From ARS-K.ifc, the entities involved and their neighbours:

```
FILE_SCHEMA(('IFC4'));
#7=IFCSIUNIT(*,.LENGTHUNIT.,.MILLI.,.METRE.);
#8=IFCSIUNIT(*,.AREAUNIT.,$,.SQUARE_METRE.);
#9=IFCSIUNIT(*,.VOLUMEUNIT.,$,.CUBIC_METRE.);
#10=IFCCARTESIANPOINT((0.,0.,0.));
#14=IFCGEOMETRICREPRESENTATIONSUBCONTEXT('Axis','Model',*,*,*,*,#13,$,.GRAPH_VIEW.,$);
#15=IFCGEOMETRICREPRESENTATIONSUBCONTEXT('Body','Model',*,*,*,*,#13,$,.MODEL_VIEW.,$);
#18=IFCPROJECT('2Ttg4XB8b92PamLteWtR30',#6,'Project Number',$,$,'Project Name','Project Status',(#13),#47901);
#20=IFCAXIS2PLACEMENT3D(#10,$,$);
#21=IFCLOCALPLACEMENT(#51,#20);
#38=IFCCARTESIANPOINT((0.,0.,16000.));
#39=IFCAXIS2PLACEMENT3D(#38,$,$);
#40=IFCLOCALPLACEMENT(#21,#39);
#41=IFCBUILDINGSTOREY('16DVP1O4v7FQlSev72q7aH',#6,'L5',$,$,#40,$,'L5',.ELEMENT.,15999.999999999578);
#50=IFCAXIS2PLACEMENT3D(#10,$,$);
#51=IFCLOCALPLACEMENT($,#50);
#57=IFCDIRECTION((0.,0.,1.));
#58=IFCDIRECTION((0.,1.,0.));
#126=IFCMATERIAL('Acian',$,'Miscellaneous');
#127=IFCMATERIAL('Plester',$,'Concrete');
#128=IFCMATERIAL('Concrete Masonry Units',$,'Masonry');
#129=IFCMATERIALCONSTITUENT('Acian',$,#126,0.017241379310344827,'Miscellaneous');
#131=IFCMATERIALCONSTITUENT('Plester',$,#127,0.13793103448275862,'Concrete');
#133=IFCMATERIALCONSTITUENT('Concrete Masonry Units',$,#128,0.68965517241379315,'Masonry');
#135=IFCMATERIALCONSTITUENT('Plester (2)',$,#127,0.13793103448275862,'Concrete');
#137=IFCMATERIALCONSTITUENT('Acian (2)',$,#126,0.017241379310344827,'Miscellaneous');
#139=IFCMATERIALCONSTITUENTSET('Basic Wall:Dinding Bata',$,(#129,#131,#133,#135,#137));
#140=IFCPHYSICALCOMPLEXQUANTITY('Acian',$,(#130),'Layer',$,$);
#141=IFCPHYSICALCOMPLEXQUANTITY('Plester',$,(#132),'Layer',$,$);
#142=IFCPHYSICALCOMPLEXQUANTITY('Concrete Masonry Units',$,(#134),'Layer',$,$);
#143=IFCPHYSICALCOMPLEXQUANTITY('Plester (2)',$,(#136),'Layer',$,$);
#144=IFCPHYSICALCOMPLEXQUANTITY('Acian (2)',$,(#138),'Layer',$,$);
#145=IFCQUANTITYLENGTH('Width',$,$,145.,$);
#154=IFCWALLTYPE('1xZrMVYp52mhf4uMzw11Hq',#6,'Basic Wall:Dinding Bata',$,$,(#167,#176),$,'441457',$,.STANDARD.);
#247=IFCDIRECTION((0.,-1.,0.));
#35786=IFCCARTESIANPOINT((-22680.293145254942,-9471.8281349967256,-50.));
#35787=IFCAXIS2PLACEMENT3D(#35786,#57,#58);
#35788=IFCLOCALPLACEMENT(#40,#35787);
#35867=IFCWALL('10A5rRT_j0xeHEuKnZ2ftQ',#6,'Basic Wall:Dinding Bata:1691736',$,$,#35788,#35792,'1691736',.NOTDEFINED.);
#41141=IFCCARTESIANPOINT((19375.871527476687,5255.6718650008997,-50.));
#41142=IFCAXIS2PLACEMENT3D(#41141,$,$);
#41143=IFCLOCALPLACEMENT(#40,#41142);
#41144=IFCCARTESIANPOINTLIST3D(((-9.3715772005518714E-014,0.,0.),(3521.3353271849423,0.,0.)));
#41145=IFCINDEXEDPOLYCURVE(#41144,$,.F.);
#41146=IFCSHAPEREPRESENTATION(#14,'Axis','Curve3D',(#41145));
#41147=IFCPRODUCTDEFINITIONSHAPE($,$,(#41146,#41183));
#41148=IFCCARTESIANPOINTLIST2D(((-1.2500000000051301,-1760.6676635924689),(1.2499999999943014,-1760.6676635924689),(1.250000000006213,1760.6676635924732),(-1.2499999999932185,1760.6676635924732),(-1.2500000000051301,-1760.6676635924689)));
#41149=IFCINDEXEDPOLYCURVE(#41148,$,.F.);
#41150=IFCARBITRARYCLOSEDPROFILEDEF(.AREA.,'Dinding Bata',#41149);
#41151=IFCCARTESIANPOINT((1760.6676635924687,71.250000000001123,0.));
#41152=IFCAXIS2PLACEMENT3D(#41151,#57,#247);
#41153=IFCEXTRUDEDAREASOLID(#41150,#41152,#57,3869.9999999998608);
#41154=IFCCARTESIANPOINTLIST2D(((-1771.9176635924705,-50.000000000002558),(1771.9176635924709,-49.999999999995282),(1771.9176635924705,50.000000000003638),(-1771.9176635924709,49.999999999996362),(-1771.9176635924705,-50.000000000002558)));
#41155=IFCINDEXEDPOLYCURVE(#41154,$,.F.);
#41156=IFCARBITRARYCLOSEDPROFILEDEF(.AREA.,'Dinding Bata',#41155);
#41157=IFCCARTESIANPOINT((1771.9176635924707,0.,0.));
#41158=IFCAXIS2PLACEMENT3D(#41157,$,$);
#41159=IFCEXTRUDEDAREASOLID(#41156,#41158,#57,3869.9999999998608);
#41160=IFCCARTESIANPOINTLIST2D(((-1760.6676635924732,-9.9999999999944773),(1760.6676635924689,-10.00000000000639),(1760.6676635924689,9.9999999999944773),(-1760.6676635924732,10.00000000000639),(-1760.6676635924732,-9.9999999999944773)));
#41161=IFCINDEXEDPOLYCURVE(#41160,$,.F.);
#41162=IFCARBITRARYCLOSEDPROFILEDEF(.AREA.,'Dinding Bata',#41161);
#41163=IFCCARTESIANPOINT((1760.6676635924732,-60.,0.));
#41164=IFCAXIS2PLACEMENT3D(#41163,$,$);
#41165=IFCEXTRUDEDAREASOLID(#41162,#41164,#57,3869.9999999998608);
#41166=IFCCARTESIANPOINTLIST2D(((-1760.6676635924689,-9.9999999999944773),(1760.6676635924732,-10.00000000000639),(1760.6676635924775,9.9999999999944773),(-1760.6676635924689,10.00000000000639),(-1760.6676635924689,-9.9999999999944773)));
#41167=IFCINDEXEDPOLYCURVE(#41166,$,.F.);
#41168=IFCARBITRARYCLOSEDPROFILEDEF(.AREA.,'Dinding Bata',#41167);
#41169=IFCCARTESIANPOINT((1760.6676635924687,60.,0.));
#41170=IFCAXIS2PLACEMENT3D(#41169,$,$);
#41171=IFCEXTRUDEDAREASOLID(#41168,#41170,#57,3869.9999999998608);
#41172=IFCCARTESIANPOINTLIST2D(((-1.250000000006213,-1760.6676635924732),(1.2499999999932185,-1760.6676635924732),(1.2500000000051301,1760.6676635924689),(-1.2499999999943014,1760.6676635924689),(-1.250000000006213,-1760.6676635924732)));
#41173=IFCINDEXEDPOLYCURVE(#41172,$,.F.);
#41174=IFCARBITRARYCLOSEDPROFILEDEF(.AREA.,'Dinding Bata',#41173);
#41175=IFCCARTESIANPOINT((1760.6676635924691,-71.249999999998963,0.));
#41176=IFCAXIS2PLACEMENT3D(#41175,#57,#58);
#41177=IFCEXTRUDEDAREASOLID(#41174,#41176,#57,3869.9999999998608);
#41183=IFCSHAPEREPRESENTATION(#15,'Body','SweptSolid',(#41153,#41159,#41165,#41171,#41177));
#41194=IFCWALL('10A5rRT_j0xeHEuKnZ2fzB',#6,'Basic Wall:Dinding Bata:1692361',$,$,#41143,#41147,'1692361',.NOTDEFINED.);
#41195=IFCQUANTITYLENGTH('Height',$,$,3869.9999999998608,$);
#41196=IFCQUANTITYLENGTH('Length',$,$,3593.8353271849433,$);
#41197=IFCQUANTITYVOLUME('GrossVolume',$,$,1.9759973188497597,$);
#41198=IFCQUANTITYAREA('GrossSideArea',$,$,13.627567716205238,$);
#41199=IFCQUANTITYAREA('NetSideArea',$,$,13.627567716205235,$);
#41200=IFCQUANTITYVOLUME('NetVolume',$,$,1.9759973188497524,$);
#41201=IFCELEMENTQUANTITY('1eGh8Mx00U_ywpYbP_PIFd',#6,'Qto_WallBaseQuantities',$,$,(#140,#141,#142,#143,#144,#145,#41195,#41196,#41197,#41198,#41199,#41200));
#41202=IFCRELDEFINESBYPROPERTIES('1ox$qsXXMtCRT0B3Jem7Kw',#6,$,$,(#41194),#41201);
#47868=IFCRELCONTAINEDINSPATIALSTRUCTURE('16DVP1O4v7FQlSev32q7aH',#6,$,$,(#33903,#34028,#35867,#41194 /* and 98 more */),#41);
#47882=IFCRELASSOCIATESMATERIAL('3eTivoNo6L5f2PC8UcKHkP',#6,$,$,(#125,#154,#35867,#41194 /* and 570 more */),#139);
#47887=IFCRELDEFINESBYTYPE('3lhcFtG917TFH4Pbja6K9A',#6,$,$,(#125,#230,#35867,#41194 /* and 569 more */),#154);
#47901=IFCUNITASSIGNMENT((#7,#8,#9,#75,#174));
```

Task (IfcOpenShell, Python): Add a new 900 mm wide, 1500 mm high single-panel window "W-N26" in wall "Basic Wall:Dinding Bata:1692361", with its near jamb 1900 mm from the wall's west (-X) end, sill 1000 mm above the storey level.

```python
import numpy as np
import ifcopenshell
import ifcopenshell.api.feature
import ifcopenshell.api.geometry
import ifcopenshell.api.pset
import ifcopenshell.api.root
import ifcopenshell.api.spatial
import ifcopenshell.geom
import ifcopenshell.util.element
import ifcopenshell.util.placement
import ifcopenshell.util.representation
import ifcopenshell.util.shape
import ifcopenshell.util.unit

model = ifcopenshell.open("ARS-K.ifc")
unit_scale = ifcopenshell.util.unit.calculate_unit_scale(model)
area_scale = ifcopenshell.util.unit.calculate_unit_scale(model, "AREAUNIT")
volume_scale = ifcopenshell.util.unit.calculate_unit_scale(model, "VOLUMEUNIT")
settings = ifcopenshell.geom.settings()


def volume(element):
    """Net volume in cubic metres, openings subtracted."""
    shape = ifcopenshell.geom.create_shape(settings, element)
    return ifcopenshell.util.shape.get_volume(shape.geometry)


wall = model.by_guid("10A5rRT_j0xeHEuKnZ2fzB")
storey = ifcopenshell.util.element.get_container(wall, ifc_class="IfcBuildingStorey")
context = ifcopenshell.util.representation.get_context(model, "Model", "Body", "MODEL_VIEW")
before = volume(wall)

width, height, from_end, sill = 0.9, 1.5, 1.9, 1  # metres

# The wall runs along its own X axis, and the end named is its -X end.
wall_shape = ifcopenshell.geom.create_shape(settings, wall)
x, y, z = ifcopenshell.util.shape.get_vertices(wall_shape.geometry).T
start = x.min() + from_end
face, thickness = float(y.min()), float(y.max() - y.min())
wall_matrix = ifcopenshell.util.placement.get_local_placement(wall.ObjectPlacement)
level = ifcopenshell.util.placement.get_local_placement(storey.ObjectPlacement)[2, 3]


def in_wall(x, y):
    """Placement at x, y metres in the wall's axes, at sill height."""
    matrix = wall_matrix.copy()
    matrix[:, 3] = wall_matrix @ np.array([x / unit_scale, y / unit_scale, 0.0, 1.0])
    matrix[2, 3] = level + sill / unit_scale
    return matrix


# Opening: a box that overshoots both wall faces by 50 mm.
opening = ifcopenshell.api.root.create_entity(model, ifc_class="IfcOpeningElement", predefined_type="OPENING")
box = ifcopenshell.api.geometry.add_wall_representation(
    model, context=context, length=width, height=height, thickness=thickness + 0.1
)
ifcopenshell.api.geometry.assign_representation(model, product=opening, representation=box)
ifcopenshell.api.geometry.edit_object_placement(model, product=opening, matrix=in_wall(start, face - 0.05), is_si=False)
ifcopenshell.api.feature.add_feature(model, feature=opening, element=wall)

window = ifcopenshell.api.root.create_entity(model, ifc_class="IfcWindow", name="W-N26", predefined_type="WINDOW")
window.OverallWidth, window.OverallHeight = width / unit_scale, height / unit_scale
window.PartitioningType = "SINGLE_PANEL"
body = ifcopenshell.api.geometry.add_window_representation(
    model,
    context=context,
    overall_width=window.OverallWidth,
    overall_height=window.OverallHeight,
    partition_type="SINGLE_PANEL",
)
ifcopenshell.api.geometry.assign_representation(model, product=window, representation=body)
ifcopenshell.api.spatial.assign_container(model, products=[window], relating_structure=storey)
ifcopenshell.api.feature.add_filling(model, opening=opening, element=window)

# Centre the window in the wall's thickness.
ifcopenshell.api.geometry.edit_object_placement(model, product=window, matrix=in_wall(start, face), is_si=False)
window_shape = ifcopenshell.geom.create_shape(settings, window)
depth = ifcopenshell.util.shape.get_vertices(window_shape.geometry)[:, 1]
offset = face + thickness / 2 - (depth.min() + depth.max()) / 2
ifcopenshell.api.geometry.edit_object_placement(model, product=window, matrix=in_wall(start, offset), is_si=False)

after = volume(wall)

# Update the wall's stored quantities.
qto = model.by_id(ifcopenshell.util.element.get_pset(wall, "Qto_WallBaseQuantities", should_inherit=False)["id"])
ifcopenshell.api.pset.edit_qto(model, qto=qto, properties={
    "NetSideArea": after / thickness / area_scale,
    "NetVolume": after / volume_scale,
})

print(f"wall volume {before:.3f} -> {after:.3f} m3")

model.write("ARS-K_rev.ifc")
```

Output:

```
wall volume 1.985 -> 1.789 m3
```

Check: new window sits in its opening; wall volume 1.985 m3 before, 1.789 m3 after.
